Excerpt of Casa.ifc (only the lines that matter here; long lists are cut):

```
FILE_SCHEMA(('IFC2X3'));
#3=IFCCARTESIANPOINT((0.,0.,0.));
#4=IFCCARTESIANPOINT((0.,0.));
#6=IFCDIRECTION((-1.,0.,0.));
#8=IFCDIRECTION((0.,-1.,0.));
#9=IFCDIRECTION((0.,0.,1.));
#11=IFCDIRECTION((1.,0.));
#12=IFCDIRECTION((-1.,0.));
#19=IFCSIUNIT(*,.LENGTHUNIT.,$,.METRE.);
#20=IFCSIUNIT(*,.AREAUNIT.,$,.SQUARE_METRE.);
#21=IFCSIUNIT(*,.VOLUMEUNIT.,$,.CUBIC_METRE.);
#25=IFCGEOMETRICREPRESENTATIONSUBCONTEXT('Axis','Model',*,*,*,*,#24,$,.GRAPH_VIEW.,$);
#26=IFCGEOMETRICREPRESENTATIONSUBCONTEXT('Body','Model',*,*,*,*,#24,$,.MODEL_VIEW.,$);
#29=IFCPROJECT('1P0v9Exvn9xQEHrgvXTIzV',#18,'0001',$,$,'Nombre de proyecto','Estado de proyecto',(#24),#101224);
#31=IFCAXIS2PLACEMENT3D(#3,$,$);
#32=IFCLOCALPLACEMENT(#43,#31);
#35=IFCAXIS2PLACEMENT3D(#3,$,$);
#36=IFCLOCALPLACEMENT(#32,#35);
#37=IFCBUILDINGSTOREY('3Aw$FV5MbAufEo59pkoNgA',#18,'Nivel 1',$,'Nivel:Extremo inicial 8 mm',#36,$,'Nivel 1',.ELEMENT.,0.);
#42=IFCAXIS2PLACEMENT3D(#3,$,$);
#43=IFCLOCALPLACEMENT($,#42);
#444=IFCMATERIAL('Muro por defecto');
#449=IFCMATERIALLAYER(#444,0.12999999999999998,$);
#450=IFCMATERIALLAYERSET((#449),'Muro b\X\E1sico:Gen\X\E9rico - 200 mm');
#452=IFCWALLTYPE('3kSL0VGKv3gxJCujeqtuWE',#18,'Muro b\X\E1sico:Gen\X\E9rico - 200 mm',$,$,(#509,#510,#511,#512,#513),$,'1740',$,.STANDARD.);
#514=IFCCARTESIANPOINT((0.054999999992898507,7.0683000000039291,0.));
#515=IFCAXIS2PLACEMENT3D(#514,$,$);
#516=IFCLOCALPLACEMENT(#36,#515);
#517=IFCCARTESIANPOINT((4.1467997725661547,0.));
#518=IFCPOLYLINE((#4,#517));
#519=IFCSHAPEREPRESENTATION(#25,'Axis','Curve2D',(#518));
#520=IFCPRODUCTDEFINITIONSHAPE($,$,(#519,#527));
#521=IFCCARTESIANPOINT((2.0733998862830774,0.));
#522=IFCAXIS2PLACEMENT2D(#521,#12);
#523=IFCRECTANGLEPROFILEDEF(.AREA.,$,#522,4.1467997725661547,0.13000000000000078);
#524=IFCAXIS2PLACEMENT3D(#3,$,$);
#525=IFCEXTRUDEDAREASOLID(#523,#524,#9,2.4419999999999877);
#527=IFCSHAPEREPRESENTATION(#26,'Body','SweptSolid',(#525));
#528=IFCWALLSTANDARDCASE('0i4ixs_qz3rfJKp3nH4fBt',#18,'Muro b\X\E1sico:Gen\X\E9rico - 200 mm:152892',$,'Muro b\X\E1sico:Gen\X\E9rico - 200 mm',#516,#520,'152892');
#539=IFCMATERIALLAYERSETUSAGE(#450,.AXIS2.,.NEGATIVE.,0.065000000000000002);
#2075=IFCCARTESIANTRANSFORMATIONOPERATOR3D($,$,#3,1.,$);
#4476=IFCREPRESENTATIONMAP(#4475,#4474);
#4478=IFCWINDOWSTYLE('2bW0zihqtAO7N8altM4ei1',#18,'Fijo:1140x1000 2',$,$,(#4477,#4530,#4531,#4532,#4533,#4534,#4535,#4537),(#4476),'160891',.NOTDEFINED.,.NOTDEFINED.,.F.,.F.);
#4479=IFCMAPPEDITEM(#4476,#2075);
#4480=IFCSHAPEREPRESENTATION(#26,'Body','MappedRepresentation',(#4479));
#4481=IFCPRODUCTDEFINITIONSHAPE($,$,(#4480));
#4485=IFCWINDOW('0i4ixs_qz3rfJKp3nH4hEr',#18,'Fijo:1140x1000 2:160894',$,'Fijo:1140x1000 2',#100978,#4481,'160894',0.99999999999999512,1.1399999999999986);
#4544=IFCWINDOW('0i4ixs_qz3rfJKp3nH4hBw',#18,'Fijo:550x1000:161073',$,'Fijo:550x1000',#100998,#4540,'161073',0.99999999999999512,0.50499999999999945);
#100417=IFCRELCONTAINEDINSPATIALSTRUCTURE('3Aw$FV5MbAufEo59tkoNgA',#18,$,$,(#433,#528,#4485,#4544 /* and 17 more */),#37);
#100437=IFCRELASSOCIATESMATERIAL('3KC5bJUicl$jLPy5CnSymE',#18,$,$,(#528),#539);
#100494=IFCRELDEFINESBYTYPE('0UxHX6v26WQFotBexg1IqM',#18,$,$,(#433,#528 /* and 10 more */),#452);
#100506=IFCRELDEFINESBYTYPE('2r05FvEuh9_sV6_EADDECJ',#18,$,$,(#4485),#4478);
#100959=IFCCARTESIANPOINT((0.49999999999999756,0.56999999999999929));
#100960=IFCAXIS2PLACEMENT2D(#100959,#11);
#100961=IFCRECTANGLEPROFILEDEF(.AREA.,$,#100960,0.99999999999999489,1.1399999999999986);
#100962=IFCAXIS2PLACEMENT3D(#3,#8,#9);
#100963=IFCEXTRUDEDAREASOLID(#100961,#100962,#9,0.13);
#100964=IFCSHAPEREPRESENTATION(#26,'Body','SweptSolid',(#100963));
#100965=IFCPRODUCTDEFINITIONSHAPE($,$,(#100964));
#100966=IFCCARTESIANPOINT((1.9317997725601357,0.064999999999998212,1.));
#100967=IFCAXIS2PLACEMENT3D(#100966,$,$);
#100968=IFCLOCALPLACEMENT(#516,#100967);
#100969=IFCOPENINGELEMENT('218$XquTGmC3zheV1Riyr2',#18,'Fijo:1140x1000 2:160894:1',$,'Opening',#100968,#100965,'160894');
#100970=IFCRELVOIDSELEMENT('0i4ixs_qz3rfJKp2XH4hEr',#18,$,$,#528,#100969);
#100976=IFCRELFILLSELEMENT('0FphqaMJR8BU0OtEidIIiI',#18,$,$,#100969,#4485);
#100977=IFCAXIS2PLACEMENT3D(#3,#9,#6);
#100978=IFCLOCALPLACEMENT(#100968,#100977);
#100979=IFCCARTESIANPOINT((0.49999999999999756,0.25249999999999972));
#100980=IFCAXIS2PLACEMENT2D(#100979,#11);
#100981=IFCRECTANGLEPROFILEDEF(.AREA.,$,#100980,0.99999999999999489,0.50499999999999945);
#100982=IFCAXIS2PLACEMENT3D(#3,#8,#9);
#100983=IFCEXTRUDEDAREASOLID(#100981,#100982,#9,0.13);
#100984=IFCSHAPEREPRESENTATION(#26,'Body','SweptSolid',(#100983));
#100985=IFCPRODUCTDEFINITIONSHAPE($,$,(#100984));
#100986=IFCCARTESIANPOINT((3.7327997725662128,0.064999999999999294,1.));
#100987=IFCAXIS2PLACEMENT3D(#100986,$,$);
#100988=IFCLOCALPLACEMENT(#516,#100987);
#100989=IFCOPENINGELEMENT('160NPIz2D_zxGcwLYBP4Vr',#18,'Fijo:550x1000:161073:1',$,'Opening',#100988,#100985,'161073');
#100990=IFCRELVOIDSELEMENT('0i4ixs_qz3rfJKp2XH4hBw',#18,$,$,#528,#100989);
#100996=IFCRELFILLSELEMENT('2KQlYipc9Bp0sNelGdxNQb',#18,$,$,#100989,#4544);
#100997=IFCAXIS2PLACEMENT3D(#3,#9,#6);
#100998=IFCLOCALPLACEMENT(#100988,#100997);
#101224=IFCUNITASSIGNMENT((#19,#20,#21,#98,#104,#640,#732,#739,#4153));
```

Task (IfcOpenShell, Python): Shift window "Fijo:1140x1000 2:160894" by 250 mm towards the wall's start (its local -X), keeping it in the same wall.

```python
import ifcopenshell
import ifcopenshell.api.geometry
import ifcopenshell.util.placement

model = ifcopenshell.open("Casa.ifc")

window = model.by_guid("0i4ixs_qz3rfJKp3nH4hEr")
opening = window.FillsVoids[0].RelatingOpeningElement
wall = opening.VoidsElements[0].RelatingBuildingElement

wall_matrix = ifcopenshell.util.placement.get_local_placement(wall.ObjectPlacement)
shift = wall_matrix[:3, 0] * -0.25
before = ifcopenshell.util.placement.get_local_placement(window.ObjectPlacement)[:3, 3].copy()

# The window is placed relative to its opening, so it follows when the opening moves.
matrix = ifcopenshell.util.placement.get_local_placement(opening.ObjectPlacement)
matrix[:3, 3] += shift
ifcopenshell.api.geometry.edit_object_placement(
    model, product=opening, matrix=matrix, is_si=False, should_transform_children=True
)

after = ifcopenshell.util.placement.get_local_placement(window.ObjectPlacement)[:3, 3]
print("window moved by", (after - before).round(3) + 0.0)

model.write("Casa_updated.ifc")
```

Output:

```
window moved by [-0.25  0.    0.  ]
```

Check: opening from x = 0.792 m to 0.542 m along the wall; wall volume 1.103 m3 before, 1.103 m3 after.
